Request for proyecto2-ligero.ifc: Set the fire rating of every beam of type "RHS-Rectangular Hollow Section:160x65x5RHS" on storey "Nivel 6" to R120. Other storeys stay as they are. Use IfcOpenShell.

First a look at what the model holds.

```python
import ifcopenshell
import ifcopenshell.util.element

model = ifcopenshell.open("proyecto2-ligero.ifc")
print(model.schema)
storey = next(s for s in model.by_type("IfcBuildingStorey") if s.Name == "Nivel 6")
beams = [e for e in ifcopenshell.util.element.get_decomposition(storey) if e.is_a("IfcBeam")]
seen = {}
for e in beams:
    element_type = ifcopenshell.util.element.get_type(e)
    key = (element_type.Name if element_type != e and element_type else None, ifcopenshell.util.element.get_pset(e, "Pset_BeamCommon", "FireRating"))
    seen[key] = seen.get(key, 0) + 1
for (name, value), count in sorted(seen.items(), key=str):
    print(count, "x", name, "|", value)
```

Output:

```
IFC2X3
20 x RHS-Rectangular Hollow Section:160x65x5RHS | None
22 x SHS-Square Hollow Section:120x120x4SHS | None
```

```python
import ifcopenshell
import ifcopenshell.api.pset
import ifcopenshell.util.element

model = ifcopenshell.open("proyecto2-ligero.ifc")

storey = next(s for s in model.by_type("IfcBuildingStorey") if s.Name == "Nivel 6")
beams = [e for e in ifcopenshell.util.element.get_decomposition(storey) if e.is_a("IfcBeam")]

count = 0
for e in beams:
    element_type = ifcopenshell.util.element.get_type(e)
    if element_type in (None, e) or element_type.Name != "RHS-Rectangular Hollow Section:160x65x5RHS":
        continue
    # add_pset returns the element's existing set when there is one.
    pset = ifcopenshell.api.pset.add_pset(model, product=e, name="Pset_BeamCommon")
    ifcopenshell.api.pset.edit_pset(model, pset=pset, properties={"FireRating": "R120"})
    count += 1

print(count, "beams updated")

model.write("proyecto2-ligero_rev.ifc")
```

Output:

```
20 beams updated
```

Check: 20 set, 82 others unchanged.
